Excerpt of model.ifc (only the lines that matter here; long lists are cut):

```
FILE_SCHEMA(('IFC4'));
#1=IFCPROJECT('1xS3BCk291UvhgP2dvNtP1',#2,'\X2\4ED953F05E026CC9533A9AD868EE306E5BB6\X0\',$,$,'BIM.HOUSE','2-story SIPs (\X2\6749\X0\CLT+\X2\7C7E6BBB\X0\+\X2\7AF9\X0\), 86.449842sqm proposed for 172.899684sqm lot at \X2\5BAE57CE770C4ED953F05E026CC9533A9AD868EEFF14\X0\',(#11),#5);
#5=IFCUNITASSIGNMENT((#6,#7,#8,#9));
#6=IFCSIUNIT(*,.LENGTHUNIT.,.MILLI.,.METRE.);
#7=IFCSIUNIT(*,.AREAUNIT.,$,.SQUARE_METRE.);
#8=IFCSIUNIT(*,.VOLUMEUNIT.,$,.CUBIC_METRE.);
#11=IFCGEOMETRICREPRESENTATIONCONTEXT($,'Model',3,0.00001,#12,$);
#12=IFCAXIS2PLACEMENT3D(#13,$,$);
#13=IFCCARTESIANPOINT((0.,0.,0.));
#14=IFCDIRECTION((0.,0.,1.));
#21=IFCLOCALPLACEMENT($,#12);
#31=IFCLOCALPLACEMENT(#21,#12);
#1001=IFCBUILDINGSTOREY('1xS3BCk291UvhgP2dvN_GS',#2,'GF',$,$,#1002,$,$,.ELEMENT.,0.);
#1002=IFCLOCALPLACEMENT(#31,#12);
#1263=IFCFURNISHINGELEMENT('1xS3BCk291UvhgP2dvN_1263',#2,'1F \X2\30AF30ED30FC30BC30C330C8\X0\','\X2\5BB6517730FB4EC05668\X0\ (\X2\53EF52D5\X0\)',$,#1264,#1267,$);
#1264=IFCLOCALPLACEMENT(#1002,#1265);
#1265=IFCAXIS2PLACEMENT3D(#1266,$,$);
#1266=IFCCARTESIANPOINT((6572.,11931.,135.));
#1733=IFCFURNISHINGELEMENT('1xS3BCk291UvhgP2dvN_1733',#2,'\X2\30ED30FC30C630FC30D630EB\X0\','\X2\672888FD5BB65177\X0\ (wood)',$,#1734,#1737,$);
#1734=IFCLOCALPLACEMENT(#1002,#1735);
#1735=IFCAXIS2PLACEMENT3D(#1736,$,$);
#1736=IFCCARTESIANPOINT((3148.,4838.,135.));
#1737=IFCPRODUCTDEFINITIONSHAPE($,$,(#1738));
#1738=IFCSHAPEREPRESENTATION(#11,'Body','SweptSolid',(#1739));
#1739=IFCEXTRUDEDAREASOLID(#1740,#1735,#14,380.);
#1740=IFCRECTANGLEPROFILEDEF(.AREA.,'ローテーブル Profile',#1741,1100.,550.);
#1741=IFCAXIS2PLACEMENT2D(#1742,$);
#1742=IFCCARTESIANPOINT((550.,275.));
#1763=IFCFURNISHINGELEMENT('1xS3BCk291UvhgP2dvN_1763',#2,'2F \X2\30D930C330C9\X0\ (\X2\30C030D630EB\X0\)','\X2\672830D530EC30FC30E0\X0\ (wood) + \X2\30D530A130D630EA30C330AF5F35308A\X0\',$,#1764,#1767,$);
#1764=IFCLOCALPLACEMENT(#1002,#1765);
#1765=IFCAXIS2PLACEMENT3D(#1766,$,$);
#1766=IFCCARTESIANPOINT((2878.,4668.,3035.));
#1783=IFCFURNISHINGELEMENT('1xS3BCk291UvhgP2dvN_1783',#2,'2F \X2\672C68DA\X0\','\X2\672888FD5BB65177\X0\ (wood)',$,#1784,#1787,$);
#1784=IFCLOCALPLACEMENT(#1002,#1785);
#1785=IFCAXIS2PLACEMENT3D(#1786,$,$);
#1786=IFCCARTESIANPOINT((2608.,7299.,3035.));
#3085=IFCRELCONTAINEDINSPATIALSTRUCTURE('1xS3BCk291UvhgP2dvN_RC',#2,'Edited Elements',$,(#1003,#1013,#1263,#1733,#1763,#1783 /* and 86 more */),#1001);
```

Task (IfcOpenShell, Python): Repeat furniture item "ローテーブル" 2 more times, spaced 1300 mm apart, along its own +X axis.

```python
import ifcopenshell
import ifcopenshell.api.geometry
import ifcopenshell.api.root
import ifcopenshell.util.element
import ifcopenshell.util.placement
import ifcopenshell.util.unit

model = ifcopenshell.open("model.ifc")
unit_scale = ifcopenshell.util.unit.calculate_unit_scale(model)


def reuse_history(source, copy):
    """copy_class also copies each property set's owner history, people and application; keep the originals."""
    for rel in copy.IsDefinedBy:
        if rel.is_a("IfcRelDefinesByProperties") and (history := rel.RelatingPropertyDefinition.OwnerHistory):
            rel.RelatingPropertyDefinition.OwnerHistory = source.OwnerHistory
            ifcopenshell.util.element.remove_deep2(model, history)


source = model.by_guid("1xS3BCk291UvhgP2dvN_1733")
base = ifcopenshell.util.placement.get_local_placement(source.ObjectPlacement)
step = base[:3, 0] * 1.3 / unit_scale

for i in range(1, 3):
    copy = ifcopenshell.api.root.copy_class(model, product=source)
    copy.Representation = ifcopenshell.util.element.copy_deep(
        model, source.Representation, exclude=["IfcGeometricRepresentationContext", "IfcRepresentationMap"]
    )
    reuse_history(source, copy)
    matrix = base.copy()
    matrix[:3, 3] += i * step
    print("added at", matrix[:3, 3].round(3) + 0.0)
    ifcopenshell.api.geometry.edit_object_placement(model, product=copy, matrix=matrix, is_si=False)

model.write("model-out.ifc")
```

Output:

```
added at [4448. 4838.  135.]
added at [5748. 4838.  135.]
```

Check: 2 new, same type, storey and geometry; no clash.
